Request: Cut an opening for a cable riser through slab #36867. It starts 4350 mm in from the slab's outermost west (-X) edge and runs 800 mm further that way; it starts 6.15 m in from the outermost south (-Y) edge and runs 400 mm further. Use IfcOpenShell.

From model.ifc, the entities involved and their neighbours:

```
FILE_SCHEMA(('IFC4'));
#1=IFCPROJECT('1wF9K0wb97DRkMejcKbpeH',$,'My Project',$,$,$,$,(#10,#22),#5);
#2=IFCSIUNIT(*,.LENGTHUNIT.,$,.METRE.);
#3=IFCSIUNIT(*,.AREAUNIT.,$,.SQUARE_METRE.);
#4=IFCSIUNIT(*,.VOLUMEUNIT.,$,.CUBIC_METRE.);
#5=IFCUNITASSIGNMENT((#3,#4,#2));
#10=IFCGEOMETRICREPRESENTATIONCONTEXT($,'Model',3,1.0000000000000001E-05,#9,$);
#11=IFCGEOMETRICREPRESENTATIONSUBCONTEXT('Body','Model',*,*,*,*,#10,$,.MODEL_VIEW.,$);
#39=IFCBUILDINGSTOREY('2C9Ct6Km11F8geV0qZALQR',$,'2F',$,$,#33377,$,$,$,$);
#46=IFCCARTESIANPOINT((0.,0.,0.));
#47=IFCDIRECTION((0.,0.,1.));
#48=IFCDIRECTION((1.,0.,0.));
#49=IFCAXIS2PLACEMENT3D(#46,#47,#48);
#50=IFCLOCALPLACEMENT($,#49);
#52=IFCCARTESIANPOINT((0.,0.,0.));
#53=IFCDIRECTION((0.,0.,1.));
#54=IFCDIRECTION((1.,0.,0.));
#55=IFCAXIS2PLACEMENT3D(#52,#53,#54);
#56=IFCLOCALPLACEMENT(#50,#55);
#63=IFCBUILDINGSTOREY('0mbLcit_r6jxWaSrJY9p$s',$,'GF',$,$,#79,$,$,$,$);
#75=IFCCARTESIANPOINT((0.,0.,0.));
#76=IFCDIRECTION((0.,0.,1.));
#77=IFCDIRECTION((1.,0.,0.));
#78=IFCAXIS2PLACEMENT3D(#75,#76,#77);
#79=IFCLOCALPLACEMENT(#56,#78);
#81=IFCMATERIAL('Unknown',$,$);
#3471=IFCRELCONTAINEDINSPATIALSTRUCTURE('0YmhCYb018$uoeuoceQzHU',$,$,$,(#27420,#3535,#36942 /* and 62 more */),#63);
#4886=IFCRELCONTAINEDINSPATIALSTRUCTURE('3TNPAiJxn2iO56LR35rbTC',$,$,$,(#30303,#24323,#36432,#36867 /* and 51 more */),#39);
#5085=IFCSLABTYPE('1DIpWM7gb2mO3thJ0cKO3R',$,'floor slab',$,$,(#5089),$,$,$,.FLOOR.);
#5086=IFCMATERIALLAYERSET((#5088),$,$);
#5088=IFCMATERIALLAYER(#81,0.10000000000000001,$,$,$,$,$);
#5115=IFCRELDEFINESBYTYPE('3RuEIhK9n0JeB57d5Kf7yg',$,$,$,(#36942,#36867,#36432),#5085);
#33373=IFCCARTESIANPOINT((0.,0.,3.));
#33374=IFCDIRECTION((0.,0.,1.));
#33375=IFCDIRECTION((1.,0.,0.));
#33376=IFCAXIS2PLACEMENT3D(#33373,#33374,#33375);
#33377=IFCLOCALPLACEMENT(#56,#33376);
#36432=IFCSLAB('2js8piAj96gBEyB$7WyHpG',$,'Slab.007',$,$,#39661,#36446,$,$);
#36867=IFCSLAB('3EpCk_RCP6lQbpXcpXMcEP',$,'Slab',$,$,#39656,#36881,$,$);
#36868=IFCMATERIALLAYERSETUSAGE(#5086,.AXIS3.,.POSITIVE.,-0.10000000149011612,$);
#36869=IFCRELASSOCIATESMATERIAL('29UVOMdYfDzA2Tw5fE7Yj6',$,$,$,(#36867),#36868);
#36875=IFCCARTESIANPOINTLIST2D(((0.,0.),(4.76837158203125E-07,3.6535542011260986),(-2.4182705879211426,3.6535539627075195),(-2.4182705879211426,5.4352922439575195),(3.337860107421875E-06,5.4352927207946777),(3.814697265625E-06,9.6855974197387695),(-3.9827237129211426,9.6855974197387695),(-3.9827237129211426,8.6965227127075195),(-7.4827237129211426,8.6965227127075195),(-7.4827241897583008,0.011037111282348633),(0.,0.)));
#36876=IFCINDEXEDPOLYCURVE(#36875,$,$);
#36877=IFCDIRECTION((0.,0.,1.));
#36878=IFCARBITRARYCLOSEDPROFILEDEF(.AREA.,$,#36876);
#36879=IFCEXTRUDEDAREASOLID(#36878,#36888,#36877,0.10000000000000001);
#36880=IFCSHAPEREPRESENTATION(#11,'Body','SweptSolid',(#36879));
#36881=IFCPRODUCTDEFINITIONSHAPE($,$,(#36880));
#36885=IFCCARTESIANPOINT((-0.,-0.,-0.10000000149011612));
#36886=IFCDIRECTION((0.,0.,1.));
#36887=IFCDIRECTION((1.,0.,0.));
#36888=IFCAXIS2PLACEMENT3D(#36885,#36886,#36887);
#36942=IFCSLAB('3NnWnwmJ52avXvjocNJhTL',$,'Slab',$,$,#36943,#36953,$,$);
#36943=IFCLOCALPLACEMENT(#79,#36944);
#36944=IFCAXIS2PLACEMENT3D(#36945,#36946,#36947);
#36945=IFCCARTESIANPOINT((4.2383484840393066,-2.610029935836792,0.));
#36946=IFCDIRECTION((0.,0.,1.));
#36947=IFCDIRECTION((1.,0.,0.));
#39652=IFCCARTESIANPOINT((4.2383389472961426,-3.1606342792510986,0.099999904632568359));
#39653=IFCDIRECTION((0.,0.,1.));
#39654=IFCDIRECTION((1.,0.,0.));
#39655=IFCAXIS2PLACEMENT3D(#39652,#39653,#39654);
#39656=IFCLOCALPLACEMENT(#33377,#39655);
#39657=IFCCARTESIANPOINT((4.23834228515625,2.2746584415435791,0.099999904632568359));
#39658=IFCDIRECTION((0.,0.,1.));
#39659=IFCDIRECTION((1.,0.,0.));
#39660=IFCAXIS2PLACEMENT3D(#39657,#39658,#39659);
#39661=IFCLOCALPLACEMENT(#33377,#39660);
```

```python
import numpy as np
import ifcopenshell
import ifcopenshell.api.feature
import ifcopenshell.api.geometry
import ifcopenshell.api.root
import ifcopenshell.geom
import ifcopenshell.util.placement
import ifcopenshell.util.representation
import ifcopenshell.util.shape
import ifcopenshell.util.unit

model = ifcopenshell.open("model.ifc")
unit_scale = ifcopenshell.util.unit.calculate_unit_scale(model)
settings = ifcopenshell.geom.settings()


def volume(element):
    """Net volume in cubic metres, openings subtracted."""
    shape = ifcopenshell.geom.create_shape(settings, element)
    return ifcopenshell.util.shape.get_volume(shape.geometry)


slab = model.by_guid("3EpCk_RCP6lQbpXcpXMcEP")
before = volume(slab)

# Extent in the slab's own axes, in metres. The edges named are its -X and -Y sides.
slab_shape = ifcopenshell.geom.create_shape(settings, slab)
vertices = ifcopenshell.util.shape.get_vertices(slab_shape.geometry)
x_min, y_min, bottom = vertices.min(axis=0)
top = vertices[:, 2].max()

opening = ifcopenshell.api.root.create_entity(model, ifc_class="IfcOpeningElement", name="Cable riser opening", predefined_type="OPENING")
context = ifcopenshell.util.representation.get_context(model, "Model", "Body", "MODEL_VIEW")
width, depth = 0.8, 0.4
outline = [(0.0, 0.0), (width, 0.0), (width, depth), (0.0, depth), (0.0, 0.0)]
# Overshoot both faces by 50 mm so the cut is clean.
shape = ifcopenshell.api.geometry.add_slab_representation(
    model, context=context, depth=top - bottom + 0.1, polyline=outline
)
ifcopenshell.api.geometry.assign_representation(model, product=opening, representation=shape)

matrix = ifcopenshell.util.placement.get_local_placement(slab.ObjectPlacement)
matrix[:, 3] = matrix @ np.append(np.array([x_min + 4.35, y_min + 6.15, bottom - 0.05]) / unit_scale, 1.0)
ifcopenshell.api.geometry.edit_object_placement(model, product=opening, matrix=matrix, is_si=False)
ifcopenshell.api.feature.add_feature(model, feature=opening, element=slab)

after = volume(slab)

print(f"slab volume {before:.3f} -> {after:.3f} m3")

model.write("model_edited.ifc")
```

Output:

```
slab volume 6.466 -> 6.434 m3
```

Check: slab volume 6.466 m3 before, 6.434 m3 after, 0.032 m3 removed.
